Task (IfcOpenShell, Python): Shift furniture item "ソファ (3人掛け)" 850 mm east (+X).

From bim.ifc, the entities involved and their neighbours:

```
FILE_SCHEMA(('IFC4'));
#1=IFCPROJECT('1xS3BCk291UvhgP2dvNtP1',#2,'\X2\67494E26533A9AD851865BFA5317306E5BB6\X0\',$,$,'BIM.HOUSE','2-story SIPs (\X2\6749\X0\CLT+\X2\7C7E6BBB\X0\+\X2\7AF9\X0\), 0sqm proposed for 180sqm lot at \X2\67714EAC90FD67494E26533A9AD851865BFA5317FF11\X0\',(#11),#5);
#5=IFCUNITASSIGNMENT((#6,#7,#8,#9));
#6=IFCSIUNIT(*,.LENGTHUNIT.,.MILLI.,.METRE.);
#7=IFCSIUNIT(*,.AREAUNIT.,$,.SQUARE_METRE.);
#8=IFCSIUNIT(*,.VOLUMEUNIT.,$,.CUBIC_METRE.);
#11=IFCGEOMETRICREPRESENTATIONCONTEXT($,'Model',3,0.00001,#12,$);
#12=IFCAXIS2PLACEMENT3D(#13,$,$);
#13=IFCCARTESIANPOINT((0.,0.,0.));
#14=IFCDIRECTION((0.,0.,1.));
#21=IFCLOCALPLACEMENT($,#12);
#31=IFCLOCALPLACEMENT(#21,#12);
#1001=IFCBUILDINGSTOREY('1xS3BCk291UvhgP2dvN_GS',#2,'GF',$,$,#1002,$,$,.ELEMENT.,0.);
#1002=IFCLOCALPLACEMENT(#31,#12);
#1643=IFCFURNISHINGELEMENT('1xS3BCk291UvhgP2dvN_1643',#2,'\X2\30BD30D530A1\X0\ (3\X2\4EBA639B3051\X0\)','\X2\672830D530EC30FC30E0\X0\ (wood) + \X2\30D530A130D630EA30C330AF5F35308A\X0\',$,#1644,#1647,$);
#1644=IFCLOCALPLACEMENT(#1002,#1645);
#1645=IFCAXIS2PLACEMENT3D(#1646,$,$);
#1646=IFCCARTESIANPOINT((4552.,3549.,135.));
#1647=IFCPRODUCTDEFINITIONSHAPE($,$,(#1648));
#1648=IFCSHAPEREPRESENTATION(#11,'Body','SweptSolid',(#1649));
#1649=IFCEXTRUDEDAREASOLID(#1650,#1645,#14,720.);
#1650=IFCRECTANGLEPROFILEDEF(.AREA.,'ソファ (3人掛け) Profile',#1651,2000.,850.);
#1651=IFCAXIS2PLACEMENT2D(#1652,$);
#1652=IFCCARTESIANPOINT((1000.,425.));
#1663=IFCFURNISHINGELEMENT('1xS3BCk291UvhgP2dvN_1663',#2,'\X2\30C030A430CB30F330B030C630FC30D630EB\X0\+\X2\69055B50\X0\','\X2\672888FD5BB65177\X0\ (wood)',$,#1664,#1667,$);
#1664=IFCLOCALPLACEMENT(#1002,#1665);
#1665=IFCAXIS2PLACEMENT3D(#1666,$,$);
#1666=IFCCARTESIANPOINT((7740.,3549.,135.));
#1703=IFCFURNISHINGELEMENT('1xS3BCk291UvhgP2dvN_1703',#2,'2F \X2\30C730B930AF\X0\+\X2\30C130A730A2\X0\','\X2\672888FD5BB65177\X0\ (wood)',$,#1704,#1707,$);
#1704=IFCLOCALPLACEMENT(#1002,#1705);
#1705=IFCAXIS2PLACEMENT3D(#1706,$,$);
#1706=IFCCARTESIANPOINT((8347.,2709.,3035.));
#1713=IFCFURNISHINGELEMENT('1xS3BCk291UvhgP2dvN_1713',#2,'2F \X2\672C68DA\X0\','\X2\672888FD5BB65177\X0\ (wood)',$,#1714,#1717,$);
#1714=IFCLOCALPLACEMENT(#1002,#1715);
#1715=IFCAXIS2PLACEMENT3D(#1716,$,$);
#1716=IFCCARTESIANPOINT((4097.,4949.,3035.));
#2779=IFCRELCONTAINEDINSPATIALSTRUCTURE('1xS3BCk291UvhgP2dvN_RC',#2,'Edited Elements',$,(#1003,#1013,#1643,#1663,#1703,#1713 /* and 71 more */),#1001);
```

```python
import ifcopenshell
import ifcopenshell.api.geometry
import ifcopenshell.util.placement

model = ifcopenshell.open("bim.ifc")

item = model.by_guid("1xS3BCk291UvhgP2dvN_1643")
matrix = ifcopenshell.util.placement.get_local_placement(item.ObjectPlacement)
matrix[0, 3] += 850.0
ifcopenshell.api.geometry.edit_object_placement(model, product=item, matrix=matrix, is_si=False)

print(ifcopenshell.util.placement.get_local_placement(item.ObjectPlacement).round(3) + 0.0)

model.write("bim_v2.ifc")
```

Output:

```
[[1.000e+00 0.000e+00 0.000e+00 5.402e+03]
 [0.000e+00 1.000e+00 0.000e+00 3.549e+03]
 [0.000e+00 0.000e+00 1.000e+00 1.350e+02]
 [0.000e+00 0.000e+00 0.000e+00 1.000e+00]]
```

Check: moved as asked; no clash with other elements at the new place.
